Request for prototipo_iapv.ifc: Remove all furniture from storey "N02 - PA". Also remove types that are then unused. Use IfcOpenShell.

First a look at what the model holds.

```python
import ifcopenshell
import ifcopenshell.util.element

model = ifcopenshell.open("prototipo_iapv.ifc")
print(model.schema)
storey = next(s for s in model.by_type("IfcBuildingStorey") if s.Name == "N02 - PA")
furniture = [e for e in ifcopenshell.util.element.get_decomposition(storey) if e.is_a("IfcFurnishingElement")]
seen = {}
for e in furniture:
    element_type = ifcopenshell.util.element.get_type(e)
    name = element_type.Name if element_type not in (None, e) else None
    seen[name] = seen.get(name, 0) + 1
for name, count in sorted(seen.items(), key=str):
    print(count, "x", name)
```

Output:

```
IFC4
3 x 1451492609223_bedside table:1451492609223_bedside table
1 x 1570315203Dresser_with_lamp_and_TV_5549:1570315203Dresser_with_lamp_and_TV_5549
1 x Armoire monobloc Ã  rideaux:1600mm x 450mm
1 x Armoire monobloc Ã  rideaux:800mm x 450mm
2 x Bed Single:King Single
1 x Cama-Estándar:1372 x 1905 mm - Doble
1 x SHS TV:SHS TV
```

```python
import ifcopenshell
import ifcopenshell.api.root
import ifcopenshell.util.element

model = ifcopenshell.open("prototipo_iapv.ifc")

storey = next(s for s in model.by_type("IfcBuildingStorey") if s.Name == "N02 - PA")
furniture = [e for e in ifcopenshell.util.element.get_decomposition(storey) if e.is_a("IfcFurnishingElement")]
types = {ifcopenshell.util.element.get_type(e) for e in furniture} - {None, *furniture}

for e in furniture:
    ifcopenshell.api.root.remove_product(model, product=e)
print(len(furniture), "removed")

unused = [t for t in types if not ifcopenshell.util.element.get_types(t)]
for t in unused:
    ifcopenshell.api.root.remove_product(model, product=t)
print(len(unused), "unused types removed")

model.write("prototipo_iapv_v2.ifc")
```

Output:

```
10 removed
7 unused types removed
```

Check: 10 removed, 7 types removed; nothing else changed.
